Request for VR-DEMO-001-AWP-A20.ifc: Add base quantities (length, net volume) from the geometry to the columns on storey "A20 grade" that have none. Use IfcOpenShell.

First a look at what the model holds.

```python
import ifcopenshell
import ifcopenshell.util.element
import ifcopenshell.util.unit

model = ifcopenshell.open("VR-DEMO-001-AWP-A20.ifc")
print(model.schema)
for unit_type in ("LENGTHUNIT", "AREAUNIT", "VOLUMEUNIT"):
    print(unit_type, ifcopenshell.util.unit.calculate_unit_scale(model, unit_type))
storey = next(s for s in model.by_type("IfcBuildingStorey") if s.Name == "A20 grade")
columns = [e for e in ifcopenshell.util.element.get_decomposition(storey) if e.is_a("IfcColumn")]
for e in sorted(columns, key=lambda e: e.id()):
    print(e.id(), e.is_a(), e.Name, list(ifcopenshell.util.element.get_psets(e, qtos_only=True)), sep=" | ")
```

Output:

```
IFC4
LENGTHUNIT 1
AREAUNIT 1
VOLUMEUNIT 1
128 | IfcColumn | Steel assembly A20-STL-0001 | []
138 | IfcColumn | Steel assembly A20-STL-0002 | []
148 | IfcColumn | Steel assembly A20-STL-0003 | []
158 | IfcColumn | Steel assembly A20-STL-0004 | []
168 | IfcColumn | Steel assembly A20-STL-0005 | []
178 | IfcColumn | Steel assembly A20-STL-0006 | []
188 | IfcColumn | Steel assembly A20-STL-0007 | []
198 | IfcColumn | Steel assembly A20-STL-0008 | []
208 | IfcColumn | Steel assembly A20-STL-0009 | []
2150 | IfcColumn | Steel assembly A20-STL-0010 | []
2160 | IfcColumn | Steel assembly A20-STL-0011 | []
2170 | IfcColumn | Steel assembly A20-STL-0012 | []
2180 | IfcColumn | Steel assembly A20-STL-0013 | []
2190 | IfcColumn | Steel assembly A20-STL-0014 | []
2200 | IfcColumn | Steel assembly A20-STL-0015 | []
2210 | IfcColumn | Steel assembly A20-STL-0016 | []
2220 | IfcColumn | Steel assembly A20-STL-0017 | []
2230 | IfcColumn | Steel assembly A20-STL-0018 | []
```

```python
import ifcopenshell
import ifcopenshell.api.pset
import ifcopenshell.geom
import ifcopenshell.util.element
import ifcopenshell.util.shape
import ifcopenshell.util.unit

model = ifcopenshell.open("VR-DEMO-001-AWP-A20.ifc")
unit_scale = ifcopenshell.util.unit.calculate_unit_scale(model)
volume_scale = ifcopenshell.util.unit.calculate_unit_scale(model, "VOLUMEUNIT")
settings = ifcopenshell.geom.settings()

storey = next(s for s in model.by_type("IfcBuildingStorey") if s.Name == "A20 grade")
columns = [e for e in ifcopenshell.util.element.get_decomposition(storey) if e.is_a("IfcColumn")]

for e in sorted(columns, key=lambda e: e.id()):
    if ifcopenshell.util.element.get_psets(e, qtos_only=True, should_inherit=False):
        continue
    # Geometry comes back in metres, in the element's own axes.
    shape = ifcopenshell.geom.create_shape(settings, e)
    values = {
        "Length": ifcopenshell.util.shape.get_z(shape.geometry) / unit_scale,
        "NetVolume": ifcopenshell.util.shape.get_volume(shape.geometry) / volume_scale,
    }
    qto = ifcopenshell.api.pset.add_qto(model, product=e, name="Qto_ColumnBaseQuantities")
    ifcopenshell.api.pset.edit_qto(model, qto=qto, properties=values)
    print(e.id(), {k: round(v, 3) for k, v in values.items()})

model.write("VR-DEMO-001-AWP-A20_updated.ifc")
```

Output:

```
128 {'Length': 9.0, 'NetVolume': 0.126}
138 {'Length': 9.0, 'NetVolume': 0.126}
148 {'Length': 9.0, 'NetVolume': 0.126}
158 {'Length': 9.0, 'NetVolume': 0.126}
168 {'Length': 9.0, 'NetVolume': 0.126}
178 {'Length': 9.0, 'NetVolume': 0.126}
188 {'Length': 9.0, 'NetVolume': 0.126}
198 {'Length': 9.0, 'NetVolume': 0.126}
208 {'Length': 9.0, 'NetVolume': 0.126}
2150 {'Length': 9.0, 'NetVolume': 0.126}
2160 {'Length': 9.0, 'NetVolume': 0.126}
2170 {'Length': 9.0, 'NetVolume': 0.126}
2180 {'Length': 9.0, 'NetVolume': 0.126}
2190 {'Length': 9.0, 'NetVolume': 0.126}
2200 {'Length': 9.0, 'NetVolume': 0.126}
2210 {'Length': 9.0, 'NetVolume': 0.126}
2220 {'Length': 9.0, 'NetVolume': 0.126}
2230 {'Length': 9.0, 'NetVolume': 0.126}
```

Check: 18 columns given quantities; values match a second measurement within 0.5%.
